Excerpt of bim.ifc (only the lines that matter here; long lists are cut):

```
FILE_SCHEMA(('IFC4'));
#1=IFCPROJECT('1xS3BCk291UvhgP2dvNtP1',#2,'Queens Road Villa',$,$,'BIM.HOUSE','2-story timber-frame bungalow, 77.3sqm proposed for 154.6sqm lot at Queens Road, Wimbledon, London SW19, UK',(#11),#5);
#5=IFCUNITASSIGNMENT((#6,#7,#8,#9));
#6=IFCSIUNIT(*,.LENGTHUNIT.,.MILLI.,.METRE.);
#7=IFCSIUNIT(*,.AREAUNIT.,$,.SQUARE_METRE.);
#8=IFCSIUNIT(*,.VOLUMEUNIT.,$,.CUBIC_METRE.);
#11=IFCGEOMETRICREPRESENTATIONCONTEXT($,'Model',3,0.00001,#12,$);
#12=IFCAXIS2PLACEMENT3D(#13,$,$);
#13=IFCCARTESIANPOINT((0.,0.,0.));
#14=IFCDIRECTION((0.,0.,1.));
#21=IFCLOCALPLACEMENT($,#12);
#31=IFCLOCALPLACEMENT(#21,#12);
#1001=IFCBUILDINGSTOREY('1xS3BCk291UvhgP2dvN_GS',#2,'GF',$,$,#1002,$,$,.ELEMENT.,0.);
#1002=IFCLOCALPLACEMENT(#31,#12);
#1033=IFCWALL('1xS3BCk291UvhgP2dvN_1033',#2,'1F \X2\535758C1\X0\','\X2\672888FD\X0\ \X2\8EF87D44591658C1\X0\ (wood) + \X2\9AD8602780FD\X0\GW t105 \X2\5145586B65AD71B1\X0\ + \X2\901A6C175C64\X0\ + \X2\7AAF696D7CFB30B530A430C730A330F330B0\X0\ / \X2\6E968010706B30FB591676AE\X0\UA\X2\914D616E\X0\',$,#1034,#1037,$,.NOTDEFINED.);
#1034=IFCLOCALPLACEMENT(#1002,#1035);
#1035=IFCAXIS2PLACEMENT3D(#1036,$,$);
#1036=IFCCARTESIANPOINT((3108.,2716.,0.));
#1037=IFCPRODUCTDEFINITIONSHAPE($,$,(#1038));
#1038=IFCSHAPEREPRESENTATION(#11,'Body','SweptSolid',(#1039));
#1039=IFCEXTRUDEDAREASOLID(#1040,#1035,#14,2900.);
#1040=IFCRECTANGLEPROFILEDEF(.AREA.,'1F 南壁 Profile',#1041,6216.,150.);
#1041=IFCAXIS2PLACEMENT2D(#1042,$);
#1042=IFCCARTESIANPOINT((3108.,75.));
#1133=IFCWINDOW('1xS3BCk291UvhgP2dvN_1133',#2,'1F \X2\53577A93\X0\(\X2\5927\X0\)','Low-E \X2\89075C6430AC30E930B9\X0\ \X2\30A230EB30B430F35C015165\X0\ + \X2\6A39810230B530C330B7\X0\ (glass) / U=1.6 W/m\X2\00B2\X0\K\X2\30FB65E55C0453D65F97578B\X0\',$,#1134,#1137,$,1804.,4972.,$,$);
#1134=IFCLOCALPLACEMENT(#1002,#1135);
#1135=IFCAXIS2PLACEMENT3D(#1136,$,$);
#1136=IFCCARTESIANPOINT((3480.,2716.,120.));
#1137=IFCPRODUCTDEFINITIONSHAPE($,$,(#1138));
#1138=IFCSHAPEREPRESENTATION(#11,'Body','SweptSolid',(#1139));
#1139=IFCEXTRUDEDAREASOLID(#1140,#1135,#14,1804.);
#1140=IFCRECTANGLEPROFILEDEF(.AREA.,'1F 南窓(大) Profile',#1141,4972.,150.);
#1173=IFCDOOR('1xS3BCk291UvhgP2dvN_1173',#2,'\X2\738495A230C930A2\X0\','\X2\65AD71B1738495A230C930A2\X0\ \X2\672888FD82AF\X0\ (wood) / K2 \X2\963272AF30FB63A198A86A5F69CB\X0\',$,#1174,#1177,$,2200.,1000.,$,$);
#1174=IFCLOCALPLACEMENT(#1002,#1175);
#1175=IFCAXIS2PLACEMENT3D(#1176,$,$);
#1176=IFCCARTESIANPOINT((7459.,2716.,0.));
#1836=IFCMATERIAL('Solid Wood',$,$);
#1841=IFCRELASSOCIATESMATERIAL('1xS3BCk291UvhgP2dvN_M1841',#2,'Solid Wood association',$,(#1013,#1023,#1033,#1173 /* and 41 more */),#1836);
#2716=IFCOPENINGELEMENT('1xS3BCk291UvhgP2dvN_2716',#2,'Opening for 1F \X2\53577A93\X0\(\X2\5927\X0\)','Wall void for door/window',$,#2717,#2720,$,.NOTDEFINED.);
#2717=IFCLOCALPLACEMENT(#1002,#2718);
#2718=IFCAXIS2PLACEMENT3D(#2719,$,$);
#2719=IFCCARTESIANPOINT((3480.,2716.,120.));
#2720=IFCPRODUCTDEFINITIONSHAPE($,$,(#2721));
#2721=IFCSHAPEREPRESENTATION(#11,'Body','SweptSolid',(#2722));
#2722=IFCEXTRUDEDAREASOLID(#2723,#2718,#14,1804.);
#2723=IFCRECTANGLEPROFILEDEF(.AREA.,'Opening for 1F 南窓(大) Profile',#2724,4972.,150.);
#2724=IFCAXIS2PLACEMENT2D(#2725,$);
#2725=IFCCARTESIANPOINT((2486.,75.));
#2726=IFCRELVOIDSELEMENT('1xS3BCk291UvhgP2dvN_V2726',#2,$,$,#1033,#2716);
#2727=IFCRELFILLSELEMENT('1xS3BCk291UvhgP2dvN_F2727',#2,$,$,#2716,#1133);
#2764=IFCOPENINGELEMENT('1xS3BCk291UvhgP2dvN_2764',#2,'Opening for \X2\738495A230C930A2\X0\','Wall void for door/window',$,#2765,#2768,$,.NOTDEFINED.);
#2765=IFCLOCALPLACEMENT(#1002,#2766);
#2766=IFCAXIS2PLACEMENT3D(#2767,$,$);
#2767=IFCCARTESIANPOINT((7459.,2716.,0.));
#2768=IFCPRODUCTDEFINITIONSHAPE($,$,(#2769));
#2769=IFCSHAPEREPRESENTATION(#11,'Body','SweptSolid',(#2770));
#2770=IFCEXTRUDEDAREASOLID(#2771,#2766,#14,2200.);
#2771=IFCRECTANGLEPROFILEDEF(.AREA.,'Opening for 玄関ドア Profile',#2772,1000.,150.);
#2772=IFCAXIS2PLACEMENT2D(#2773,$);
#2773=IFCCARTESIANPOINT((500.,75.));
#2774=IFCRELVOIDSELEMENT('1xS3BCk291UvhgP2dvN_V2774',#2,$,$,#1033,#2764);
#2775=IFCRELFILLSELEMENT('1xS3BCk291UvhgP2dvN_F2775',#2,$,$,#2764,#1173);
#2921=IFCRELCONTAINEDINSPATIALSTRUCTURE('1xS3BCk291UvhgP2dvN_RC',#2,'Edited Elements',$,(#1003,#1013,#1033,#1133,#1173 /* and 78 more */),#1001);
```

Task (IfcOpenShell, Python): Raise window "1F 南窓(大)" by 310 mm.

```python
import numpy as np
import ifcopenshell
import ifcopenshell.api.geometry
import ifcopenshell.util.placement
import ifcopenshell.util.unit

model = ifcopenshell.open("bim.ifc")
unit_scale = ifcopenshell.util.unit.calculate_unit_scale(model)

window = model.by_guid("1xS3BCk291UvhgP2dvN_1133")
opening = window.FillsVoids[0].RelatingOpeningElement
dz = 0.31 / unit_scale

shift = np.array([0.0, 0.0, dz])
# The window is not placed relative to its opening, so move both.
for product in (opening, window):
    matrix = ifcopenshell.util.placement.get_local_placement(product.ObjectPlacement)
    matrix[:3, 3] += shift
    ifcopenshell.api.geometry.edit_object_placement(model, product=product, matrix=matrix, is_si=False)

print(f"moved by {dz * unit_scale:+.3f} m")

model.write("bim_edited.ifc")
```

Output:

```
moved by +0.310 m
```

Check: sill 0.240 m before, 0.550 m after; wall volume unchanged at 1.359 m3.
